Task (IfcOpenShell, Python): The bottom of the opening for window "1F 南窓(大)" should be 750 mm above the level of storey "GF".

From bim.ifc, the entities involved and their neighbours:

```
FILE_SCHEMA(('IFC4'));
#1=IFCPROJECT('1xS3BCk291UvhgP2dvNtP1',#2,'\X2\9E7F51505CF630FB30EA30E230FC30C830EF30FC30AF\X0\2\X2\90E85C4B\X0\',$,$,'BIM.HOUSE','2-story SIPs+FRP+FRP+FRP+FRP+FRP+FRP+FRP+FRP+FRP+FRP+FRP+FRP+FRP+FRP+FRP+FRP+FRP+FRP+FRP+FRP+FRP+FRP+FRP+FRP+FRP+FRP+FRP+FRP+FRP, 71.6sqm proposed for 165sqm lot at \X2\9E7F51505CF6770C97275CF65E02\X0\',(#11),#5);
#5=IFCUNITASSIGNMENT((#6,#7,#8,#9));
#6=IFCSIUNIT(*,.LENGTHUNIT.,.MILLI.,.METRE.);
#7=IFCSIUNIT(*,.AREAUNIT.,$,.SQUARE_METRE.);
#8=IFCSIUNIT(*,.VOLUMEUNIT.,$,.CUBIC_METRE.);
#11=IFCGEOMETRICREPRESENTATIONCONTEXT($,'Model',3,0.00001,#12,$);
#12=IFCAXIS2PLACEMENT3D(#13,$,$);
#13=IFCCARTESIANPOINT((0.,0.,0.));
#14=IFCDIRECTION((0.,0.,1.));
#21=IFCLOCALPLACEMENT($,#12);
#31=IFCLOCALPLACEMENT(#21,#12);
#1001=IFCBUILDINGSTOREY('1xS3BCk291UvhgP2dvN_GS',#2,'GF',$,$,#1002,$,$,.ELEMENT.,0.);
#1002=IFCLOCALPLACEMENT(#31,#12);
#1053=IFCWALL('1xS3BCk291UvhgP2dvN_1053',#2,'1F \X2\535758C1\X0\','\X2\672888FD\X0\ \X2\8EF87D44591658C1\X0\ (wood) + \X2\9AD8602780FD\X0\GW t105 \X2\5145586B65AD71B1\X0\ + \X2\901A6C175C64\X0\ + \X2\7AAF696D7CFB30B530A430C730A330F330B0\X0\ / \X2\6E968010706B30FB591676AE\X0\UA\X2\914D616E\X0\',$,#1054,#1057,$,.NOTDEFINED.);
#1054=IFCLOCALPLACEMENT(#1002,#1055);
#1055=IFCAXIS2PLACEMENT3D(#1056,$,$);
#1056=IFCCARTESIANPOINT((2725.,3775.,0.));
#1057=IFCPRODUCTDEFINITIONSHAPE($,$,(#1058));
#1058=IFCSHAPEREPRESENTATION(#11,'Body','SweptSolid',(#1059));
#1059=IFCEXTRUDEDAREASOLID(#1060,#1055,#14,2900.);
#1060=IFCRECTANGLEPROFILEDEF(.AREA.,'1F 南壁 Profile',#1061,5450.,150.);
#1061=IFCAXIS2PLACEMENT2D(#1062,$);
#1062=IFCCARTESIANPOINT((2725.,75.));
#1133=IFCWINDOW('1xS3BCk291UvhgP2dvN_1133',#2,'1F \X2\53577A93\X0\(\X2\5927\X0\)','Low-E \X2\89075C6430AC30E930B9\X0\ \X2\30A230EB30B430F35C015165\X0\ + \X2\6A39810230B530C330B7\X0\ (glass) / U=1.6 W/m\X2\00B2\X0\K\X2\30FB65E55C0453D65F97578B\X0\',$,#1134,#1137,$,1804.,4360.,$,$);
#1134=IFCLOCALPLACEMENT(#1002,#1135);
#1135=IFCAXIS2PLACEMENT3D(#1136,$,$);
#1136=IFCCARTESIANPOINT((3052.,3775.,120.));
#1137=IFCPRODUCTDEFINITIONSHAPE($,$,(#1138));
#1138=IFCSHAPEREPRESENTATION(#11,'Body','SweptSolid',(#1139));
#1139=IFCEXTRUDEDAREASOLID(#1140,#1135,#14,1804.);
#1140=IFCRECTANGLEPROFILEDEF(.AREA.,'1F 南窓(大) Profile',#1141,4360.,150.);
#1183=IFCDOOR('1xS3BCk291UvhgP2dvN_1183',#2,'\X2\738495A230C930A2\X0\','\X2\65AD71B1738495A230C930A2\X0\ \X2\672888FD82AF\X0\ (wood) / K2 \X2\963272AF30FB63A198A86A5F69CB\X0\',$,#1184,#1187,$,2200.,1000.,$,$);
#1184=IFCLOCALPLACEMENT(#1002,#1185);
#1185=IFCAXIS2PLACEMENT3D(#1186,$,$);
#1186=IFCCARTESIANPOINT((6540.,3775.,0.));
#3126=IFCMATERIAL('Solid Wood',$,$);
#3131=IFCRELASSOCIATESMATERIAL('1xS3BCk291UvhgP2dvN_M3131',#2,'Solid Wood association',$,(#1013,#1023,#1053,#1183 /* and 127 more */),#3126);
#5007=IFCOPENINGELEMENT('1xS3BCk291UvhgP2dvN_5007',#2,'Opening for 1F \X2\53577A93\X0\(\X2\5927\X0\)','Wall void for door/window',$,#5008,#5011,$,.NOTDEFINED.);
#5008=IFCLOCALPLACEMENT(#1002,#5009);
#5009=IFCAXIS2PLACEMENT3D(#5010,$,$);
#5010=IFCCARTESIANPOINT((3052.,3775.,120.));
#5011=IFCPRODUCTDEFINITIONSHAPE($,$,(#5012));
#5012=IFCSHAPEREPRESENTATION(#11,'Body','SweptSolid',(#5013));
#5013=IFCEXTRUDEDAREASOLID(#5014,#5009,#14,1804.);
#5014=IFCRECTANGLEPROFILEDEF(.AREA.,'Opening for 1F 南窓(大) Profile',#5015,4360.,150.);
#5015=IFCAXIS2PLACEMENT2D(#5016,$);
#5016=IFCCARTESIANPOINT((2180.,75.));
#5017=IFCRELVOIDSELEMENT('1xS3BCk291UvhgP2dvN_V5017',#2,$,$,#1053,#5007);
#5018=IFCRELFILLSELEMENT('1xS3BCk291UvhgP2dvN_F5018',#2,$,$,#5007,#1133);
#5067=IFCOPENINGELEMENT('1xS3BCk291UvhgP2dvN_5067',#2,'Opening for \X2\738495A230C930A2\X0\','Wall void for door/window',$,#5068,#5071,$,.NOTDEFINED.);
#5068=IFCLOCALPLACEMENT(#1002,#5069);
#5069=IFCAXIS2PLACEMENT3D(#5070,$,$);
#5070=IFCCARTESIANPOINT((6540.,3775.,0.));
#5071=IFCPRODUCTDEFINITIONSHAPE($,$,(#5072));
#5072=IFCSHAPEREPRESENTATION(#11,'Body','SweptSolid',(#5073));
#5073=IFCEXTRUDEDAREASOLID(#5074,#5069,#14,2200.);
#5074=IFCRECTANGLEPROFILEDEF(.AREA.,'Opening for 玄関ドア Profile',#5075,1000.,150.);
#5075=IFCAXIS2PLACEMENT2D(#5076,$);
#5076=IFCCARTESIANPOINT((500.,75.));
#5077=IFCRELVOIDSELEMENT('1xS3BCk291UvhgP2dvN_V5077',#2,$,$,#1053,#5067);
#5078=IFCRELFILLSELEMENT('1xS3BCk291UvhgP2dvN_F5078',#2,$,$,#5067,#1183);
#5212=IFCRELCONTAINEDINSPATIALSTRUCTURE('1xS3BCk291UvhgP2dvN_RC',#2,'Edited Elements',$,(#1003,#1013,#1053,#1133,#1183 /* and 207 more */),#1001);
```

```python
import numpy as np
import ifcopenshell
import ifcopenshell.api.geometry
import ifcopenshell.geom
import ifcopenshell.util.element
import ifcopenshell.util.placement
import ifcopenshell.util.shape
import ifcopenshell.util.unit

model = ifcopenshell.open("bim.ifc")
unit_scale = ifcopenshell.util.unit.calculate_unit_scale(model)

window = model.by_guid("1xS3BCk291UvhgP2dvN_1133")
opening = window.FillsVoids[0].RelatingOpeningElement
storey = ifcopenshell.util.element.get_container(window, ifc_class="IfcBuildingStorey")
level = ifcopenshell.util.placement.get_local_placement(storey.ObjectPlacement)[2, 3]

# The opening's origin need not be at the sill, so measure its lowest point.
shape = ifcopenshell.geom.create_shape(ifcopenshell.geom.settings(), opening)
bottom = ifcopenshell.util.shape.get_shape_bottom_elevation(shape, shape.geometry) / unit_scale
dz = level + 750.0 - bottom

shift = np.array([0.0, 0.0, dz])
# The window is not placed relative to its opening, so move both.
for product in (opening, window):
    matrix = ifcopenshell.util.placement.get_local_placement(product.ObjectPlacement)
    matrix[:3, 3] += shift
    ifcopenshell.api.geometry.edit_object_placement(model, product=product, matrix=matrix, is_si=False)

print(f"moved by {dz * unit_scale:+.3f} m")

model.write("bim_updated.ifc")
```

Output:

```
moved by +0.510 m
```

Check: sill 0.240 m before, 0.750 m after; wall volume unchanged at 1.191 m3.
